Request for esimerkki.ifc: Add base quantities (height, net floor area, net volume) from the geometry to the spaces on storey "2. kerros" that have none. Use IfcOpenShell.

First a look at what the model holds.

```python
import ifcopenshell
import ifcopenshell.util.element
import ifcopenshell.util.unit

model = ifcopenshell.open("esimerkki.ifc")
print(model.schema)
for unit_type in ("LENGTHUNIT", "AREAUNIT", "VOLUMEUNIT"):
    print(unit_type, ifcopenshell.util.unit.calculate_unit_scale(model, unit_type))
storey = next(s for s in model.by_type("IfcBuildingStorey") if s.Name == "2. kerros")
spaces = [e for e in ifcopenshell.util.element.get_decomposition(storey) if e.is_a("IfcSpace")]
for e in sorted(spaces, key=lambda e: e.id()):
    print(e.id(), e.is_a(), e.Name, list(ifcopenshell.util.element.get_psets(e, qtos_only=True)), sep=" | ")
```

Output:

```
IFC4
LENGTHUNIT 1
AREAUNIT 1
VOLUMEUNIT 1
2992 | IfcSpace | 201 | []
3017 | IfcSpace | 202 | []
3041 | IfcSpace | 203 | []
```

```python
import ifcopenshell
import ifcopenshell.api.pset
import ifcopenshell.geom
import ifcopenshell.util.element
import ifcopenshell.util.shape
import ifcopenshell.util.unit

model = ifcopenshell.open("esimerkki.ifc")
unit_scale = ifcopenshell.util.unit.calculate_unit_scale(model)
area_scale = ifcopenshell.util.unit.calculate_unit_scale(model, "AREAUNIT")
volume_scale = ifcopenshell.util.unit.calculate_unit_scale(model, "VOLUMEUNIT")
settings = ifcopenshell.geom.settings()

storey = next(s for s in model.by_type("IfcBuildingStorey") if s.Name == "2. kerros")
spaces = [e for e in ifcopenshell.util.element.get_decomposition(storey) if e.is_a("IfcSpace")]

for e in sorted(spaces, key=lambda e: e.id()):
    if ifcopenshell.util.element.get_psets(e, qtos_only=True, should_inherit=False):
        continue
    # Geometry comes back in metres, in the element's own axes.
    shape = ifcopenshell.geom.create_shape(settings, e)
    values = {
        "Height": ifcopenshell.util.shape.get_z(shape.geometry) / unit_scale,
        "NetFloorArea": ifcopenshell.util.shape.get_footprint_area(shape.geometry) / area_scale,
        "NetVolume": ifcopenshell.util.shape.get_volume(shape.geometry) / volume_scale,
    }
    qto = ifcopenshell.api.pset.add_qto(model, product=e, name="Qto_SpaceBaseQuantities")
    ifcopenshell.api.pset.edit_qto(model, qto=qto, properties=values)
    print(e.id(), {k: round(v, 3) for k, v in values.items()})

model.write("esimerkki_edited.ifc")
```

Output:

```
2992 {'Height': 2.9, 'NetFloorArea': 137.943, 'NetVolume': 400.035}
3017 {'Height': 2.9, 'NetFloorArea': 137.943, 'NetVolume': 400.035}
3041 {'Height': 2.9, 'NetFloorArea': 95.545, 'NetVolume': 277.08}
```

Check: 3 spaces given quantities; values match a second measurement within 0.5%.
